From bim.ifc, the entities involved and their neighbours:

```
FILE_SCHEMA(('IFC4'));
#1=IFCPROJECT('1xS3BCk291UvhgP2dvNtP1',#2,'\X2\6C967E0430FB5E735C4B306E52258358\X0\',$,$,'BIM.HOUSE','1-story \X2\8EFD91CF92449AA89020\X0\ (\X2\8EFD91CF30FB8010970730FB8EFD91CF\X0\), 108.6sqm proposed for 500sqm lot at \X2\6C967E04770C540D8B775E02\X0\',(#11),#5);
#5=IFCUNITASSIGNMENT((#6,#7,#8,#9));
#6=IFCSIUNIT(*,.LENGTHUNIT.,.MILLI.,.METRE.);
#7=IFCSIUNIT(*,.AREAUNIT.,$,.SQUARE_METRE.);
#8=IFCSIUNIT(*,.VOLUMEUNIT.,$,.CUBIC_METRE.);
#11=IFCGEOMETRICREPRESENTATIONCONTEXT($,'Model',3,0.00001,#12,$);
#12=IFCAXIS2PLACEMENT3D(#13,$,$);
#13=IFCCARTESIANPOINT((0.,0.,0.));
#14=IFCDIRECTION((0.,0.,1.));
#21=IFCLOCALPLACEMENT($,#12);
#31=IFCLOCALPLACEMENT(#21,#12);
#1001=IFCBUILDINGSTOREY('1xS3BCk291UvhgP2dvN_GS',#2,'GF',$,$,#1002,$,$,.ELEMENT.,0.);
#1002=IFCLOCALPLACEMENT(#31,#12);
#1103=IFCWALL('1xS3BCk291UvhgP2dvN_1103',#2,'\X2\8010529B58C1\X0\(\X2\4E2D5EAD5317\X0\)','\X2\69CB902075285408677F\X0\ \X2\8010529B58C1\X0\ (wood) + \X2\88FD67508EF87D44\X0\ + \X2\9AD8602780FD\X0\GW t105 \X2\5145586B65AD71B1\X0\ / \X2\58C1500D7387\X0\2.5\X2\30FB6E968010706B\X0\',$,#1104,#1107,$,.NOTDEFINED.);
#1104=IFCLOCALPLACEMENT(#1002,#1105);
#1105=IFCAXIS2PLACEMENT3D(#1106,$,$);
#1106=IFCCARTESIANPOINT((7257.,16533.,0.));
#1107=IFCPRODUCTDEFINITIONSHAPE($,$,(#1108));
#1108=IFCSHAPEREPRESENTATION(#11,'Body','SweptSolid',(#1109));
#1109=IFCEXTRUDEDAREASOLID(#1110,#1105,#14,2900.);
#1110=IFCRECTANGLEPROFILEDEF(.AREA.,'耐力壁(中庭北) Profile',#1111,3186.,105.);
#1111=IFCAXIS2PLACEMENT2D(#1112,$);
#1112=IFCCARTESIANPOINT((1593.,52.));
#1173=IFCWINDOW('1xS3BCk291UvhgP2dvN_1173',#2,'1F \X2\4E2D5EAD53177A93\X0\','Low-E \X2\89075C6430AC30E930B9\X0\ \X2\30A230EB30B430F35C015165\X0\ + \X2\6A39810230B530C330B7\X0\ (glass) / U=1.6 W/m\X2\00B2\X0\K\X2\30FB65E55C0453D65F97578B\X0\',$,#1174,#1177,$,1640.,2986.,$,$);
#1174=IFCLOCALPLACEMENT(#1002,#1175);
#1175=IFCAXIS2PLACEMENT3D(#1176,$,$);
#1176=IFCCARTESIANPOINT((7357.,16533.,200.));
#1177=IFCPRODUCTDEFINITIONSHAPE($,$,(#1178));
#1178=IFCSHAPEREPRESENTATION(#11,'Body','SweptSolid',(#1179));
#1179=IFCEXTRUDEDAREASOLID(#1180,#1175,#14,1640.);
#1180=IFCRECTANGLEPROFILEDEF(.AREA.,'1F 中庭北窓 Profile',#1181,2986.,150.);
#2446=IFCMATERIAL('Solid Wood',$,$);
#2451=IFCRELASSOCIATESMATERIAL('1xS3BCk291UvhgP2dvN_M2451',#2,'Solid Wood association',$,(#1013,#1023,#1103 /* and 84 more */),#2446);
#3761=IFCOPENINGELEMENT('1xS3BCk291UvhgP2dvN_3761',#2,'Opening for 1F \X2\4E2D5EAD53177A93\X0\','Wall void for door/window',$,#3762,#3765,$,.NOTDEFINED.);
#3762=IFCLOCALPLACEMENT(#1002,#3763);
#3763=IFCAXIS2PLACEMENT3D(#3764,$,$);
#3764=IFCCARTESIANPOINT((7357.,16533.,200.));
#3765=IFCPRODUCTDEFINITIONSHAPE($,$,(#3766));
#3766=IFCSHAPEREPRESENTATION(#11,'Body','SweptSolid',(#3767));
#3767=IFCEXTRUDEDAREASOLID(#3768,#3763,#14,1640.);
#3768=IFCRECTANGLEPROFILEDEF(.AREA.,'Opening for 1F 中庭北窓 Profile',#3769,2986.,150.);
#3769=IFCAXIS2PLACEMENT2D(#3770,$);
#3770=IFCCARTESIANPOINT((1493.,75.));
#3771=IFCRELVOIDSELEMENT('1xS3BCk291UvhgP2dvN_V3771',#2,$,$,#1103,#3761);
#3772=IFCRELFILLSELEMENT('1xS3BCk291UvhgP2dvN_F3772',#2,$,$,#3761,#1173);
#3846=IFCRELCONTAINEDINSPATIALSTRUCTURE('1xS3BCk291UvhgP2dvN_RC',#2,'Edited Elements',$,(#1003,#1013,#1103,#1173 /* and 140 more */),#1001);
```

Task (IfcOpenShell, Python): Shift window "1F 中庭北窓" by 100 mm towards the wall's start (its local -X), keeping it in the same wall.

```python
import ifcopenshell
import ifcopenshell.api.geometry
import ifcopenshell.util.placement
import ifcopenshell.util.unit

model = ifcopenshell.open("bim.ifc")
unit_scale = ifcopenshell.util.unit.calculate_unit_scale(model)

window = model.by_guid("1xS3BCk291UvhgP2dvN_1173")
opening = window.FillsVoids[0].RelatingOpeningElement
wall = opening.VoidsElements[0].RelatingBuildingElement

wall_matrix = ifcopenshell.util.placement.get_local_placement(wall.ObjectPlacement)
shift = wall_matrix[:3, 0] * -0.1 / unit_scale
before = ifcopenshell.util.placement.get_local_placement(window.ObjectPlacement)[:3, 3].copy()

# The window is not placed relative to its opening, so move both.
for product in (opening, window):
    matrix = ifcopenshell.util.placement.get_local_placement(product.ObjectPlacement)
    matrix[:3, 3] += shift
    ifcopenshell.api.geometry.edit_object_placement(model, product=product, matrix=matrix, is_si=False)

after = ifcopenshell.util.placement.get_local_placement(window.ObjectPlacement)[:3, 3]
print("window moved by", (after - before).round(3) + 0.0)

model.write("bim_rev.ifc")
```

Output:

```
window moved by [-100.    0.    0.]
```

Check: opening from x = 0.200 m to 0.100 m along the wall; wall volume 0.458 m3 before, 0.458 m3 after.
